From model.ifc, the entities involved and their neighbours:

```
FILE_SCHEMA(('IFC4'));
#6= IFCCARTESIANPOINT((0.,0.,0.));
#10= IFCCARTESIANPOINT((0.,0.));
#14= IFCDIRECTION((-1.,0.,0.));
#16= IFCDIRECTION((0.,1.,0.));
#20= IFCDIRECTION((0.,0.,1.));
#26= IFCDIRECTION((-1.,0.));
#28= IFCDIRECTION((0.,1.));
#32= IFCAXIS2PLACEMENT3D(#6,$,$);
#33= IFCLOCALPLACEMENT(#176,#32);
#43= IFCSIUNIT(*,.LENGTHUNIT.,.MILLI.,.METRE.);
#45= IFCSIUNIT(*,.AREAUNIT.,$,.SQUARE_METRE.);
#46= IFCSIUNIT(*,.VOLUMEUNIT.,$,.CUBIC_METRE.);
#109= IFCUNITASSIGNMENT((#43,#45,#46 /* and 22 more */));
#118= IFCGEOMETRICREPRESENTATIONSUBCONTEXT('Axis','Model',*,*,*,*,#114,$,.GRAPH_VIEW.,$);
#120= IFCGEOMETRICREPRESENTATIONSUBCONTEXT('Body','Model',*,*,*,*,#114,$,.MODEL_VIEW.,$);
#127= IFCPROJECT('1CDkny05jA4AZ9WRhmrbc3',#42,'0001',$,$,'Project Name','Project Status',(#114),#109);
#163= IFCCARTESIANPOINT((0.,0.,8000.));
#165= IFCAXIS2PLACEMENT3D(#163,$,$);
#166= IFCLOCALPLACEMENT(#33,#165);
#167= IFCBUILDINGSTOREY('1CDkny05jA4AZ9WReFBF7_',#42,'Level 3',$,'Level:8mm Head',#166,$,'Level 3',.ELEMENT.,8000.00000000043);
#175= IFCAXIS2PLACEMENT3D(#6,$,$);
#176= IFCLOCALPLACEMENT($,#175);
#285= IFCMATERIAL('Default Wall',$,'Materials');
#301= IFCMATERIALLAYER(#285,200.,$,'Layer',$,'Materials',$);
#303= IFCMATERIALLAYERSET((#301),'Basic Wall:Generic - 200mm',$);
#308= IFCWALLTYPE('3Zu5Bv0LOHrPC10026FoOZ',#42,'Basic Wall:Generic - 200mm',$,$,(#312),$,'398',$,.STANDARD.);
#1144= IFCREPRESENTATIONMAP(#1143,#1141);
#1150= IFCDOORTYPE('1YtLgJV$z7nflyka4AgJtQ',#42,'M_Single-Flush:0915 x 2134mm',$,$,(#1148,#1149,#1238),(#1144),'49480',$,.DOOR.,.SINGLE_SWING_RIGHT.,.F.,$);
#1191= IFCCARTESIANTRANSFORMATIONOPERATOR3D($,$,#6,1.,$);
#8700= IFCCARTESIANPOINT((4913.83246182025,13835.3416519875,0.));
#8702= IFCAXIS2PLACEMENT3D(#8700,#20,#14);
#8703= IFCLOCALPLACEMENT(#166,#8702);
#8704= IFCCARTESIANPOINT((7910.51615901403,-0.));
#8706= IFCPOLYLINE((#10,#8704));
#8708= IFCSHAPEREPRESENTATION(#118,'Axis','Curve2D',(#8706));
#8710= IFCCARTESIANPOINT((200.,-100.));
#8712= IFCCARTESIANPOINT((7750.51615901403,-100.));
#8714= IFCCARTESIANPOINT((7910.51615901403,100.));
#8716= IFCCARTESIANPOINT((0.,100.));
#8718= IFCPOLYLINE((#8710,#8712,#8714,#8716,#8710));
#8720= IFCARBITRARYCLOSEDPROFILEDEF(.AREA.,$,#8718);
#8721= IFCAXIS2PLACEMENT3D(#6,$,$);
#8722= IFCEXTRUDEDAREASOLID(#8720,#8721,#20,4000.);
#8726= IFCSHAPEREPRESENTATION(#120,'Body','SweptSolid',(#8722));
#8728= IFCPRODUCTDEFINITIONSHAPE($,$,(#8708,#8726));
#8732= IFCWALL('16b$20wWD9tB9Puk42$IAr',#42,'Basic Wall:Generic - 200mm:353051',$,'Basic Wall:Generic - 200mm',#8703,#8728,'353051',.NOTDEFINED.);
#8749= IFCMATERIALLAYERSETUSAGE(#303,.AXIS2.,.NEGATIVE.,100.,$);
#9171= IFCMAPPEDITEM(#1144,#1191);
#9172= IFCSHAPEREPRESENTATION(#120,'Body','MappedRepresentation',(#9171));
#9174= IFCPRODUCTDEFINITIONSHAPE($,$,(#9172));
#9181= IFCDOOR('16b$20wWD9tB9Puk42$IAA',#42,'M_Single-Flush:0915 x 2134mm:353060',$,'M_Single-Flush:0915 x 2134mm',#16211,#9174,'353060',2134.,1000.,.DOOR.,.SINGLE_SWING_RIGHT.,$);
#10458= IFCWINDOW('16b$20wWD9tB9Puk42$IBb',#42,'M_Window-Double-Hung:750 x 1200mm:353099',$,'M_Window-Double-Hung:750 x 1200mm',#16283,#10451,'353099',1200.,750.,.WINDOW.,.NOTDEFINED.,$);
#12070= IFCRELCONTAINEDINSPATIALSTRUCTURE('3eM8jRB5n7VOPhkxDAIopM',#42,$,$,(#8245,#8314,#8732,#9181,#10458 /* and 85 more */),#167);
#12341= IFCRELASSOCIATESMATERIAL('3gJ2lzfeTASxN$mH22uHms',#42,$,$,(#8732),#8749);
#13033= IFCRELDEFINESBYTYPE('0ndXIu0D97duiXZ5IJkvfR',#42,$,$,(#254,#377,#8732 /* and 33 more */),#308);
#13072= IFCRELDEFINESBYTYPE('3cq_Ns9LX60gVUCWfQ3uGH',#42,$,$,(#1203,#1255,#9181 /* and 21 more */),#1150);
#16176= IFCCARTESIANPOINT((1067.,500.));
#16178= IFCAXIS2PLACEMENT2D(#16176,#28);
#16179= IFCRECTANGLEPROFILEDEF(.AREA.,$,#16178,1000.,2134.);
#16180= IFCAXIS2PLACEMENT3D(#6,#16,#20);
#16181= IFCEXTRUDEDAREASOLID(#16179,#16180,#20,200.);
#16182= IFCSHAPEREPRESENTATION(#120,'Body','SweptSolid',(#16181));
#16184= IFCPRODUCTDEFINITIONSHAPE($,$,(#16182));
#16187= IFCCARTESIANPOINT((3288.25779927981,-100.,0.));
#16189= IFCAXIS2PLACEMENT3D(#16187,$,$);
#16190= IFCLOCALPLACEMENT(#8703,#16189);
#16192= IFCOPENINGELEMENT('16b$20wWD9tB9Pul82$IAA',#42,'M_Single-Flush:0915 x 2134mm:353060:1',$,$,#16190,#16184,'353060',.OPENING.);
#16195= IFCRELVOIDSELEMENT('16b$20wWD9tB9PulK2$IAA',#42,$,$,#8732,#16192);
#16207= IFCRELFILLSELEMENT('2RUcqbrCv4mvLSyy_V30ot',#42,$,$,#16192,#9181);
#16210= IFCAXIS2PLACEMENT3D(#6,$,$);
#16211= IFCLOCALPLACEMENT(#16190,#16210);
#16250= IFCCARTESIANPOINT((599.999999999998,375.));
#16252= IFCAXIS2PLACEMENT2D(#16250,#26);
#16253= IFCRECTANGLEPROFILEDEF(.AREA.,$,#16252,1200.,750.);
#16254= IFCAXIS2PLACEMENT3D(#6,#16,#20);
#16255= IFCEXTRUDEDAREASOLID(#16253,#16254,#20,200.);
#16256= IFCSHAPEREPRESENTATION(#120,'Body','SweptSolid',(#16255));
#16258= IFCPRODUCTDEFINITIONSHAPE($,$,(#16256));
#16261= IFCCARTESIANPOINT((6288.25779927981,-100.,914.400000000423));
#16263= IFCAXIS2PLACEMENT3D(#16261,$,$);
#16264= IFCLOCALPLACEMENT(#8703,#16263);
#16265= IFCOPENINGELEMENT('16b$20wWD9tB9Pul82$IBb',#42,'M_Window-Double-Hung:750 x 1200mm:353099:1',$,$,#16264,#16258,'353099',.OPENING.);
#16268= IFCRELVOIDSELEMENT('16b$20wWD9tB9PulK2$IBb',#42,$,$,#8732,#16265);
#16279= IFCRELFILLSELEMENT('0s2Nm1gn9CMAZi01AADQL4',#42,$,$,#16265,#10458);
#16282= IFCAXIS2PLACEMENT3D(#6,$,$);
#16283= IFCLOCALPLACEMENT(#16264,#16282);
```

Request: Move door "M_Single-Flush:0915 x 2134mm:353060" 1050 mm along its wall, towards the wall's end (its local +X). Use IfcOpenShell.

```python
import ifcopenshell
import ifcopenshell.api.geometry
import ifcopenshell.util.placement
import ifcopenshell.util.unit

model = ifcopenshell.open("model.ifc")
unit_scale = ifcopenshell.util.unit.calculate_unit_scale(model)

door = model.by_guid("16b$20wWD9tB9Puk42$IAA")
opening = door.FillsVoids[0].RelatingOpeningElement
wall = opening.VoidsElements[0].RelatingBuildingElement

wall_matrix = ifcopenshell.util.placement.get_local_placement(wall.ObjectPlacement)
shift = wall_matrix[:3, 0] * 1.05 / unit_scale
before = ifcopenshell.util.placement.get_local_placement(door.ObjectPlacement)[:3, 3].copy()

# The door is placed relative to its opening, so it follows when the opening moves.
matrix = ifcopenshell.util.placement.get_local_placement(opening.ObjectPlacement)
matrix[:3, 3] += shift
ifcopenshell.api.geometry.edit_object_placement(
    model, product=opening, matrix=matrix, is_si=False, should_transform_children=True
)

after = ifcopenshell.util.placement.get_local_placement(door.ObjectPlacement)[:3, 3]
print("door moved by", (after - before).round(3) + 0.0)

model.write("model_v2.ifc")
```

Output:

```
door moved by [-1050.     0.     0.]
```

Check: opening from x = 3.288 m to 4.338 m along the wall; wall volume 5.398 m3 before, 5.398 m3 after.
